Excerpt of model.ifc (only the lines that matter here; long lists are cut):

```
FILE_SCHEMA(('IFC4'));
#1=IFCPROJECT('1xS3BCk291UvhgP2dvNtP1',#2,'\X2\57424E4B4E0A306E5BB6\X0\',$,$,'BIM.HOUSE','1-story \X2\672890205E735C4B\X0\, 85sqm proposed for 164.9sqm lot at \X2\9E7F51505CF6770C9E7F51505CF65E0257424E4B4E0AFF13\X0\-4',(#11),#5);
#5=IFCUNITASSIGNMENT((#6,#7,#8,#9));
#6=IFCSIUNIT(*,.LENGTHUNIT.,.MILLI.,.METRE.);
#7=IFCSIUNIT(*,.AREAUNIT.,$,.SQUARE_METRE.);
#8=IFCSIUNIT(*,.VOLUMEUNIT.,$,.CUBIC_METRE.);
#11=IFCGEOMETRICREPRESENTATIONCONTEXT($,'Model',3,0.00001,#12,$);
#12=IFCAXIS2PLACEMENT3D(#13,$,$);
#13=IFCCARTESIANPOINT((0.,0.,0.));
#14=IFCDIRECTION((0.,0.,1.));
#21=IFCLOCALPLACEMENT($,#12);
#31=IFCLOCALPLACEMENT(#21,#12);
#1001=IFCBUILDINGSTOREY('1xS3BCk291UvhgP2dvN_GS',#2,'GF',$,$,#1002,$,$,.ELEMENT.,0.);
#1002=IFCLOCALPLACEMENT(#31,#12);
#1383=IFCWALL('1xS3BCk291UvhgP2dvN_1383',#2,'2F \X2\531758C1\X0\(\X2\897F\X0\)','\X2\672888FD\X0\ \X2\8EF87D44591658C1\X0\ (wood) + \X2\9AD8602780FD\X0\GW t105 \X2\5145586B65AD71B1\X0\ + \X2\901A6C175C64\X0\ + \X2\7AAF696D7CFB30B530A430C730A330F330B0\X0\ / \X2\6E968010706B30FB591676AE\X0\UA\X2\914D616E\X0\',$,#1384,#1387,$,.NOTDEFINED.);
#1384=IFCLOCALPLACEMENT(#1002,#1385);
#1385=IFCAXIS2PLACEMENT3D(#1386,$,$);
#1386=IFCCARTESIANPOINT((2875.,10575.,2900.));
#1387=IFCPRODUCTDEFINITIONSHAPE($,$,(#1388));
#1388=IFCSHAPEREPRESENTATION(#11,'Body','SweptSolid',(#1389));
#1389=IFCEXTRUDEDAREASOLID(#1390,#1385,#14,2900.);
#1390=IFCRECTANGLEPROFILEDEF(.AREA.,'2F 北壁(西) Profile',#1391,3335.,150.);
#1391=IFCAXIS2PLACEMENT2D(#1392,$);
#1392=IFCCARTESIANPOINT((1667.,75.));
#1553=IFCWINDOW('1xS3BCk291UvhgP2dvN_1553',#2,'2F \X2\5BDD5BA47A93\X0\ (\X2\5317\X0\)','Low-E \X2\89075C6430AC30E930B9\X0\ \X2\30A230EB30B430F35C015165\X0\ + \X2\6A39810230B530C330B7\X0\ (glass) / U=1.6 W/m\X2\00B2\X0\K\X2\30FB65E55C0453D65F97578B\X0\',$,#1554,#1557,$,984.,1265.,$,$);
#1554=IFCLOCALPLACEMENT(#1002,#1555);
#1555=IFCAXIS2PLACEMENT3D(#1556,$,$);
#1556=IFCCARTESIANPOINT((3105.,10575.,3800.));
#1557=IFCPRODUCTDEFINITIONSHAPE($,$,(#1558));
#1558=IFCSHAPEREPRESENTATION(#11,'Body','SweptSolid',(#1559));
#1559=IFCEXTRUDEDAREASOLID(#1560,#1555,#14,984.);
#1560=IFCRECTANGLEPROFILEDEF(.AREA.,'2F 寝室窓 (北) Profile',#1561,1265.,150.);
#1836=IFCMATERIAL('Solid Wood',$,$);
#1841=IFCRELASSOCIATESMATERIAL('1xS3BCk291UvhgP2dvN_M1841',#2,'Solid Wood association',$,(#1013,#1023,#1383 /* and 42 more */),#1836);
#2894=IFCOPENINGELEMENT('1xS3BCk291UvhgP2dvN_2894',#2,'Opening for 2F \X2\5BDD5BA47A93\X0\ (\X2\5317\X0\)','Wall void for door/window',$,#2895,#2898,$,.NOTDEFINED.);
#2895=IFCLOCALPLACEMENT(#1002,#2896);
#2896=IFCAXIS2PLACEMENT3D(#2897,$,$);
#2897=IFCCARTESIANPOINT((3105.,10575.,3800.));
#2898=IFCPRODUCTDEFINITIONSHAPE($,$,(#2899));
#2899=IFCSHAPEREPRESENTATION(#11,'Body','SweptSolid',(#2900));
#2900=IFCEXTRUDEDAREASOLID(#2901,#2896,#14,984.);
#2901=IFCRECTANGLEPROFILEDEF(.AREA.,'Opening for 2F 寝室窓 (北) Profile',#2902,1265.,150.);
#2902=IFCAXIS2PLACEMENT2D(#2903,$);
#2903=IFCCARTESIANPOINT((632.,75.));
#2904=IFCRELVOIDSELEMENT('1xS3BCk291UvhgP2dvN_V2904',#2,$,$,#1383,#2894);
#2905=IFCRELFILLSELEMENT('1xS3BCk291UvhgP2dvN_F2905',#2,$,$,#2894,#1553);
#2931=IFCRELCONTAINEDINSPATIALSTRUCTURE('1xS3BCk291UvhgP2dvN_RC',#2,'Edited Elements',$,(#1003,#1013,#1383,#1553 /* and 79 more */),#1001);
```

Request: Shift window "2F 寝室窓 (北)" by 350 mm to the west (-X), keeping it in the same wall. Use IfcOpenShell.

```python
import ifcopenshell
import ifcopenshell.api.geometry
import ifcopenshell.util.placement

model = ifcopenshell.open("model.ifc")

window = model.by_guid("1xS3BCk291UvhgP2dvN_1553")
opening = window.FillsVoids[0].RelatingOpeningElement
wall = opening.VoidsElements[0].RelatingBuildingElement

wall_matrix = ifcopenshell.util.placement.get_local_placement(wall.ObjectPlacement)
shift = wall_matrix[:3, 0] * -350.0
before = ifcopenshell.util.placement.get_local_placement(window.ObjectPlacement)[:3, 3].copy()

# The window is not placed relative to its opening, so move both.
for product in (opening, window):
    matrix = ifcopenshell.util.placement.get_local_placement(product.ObjectPlacement)
    matrix[:3, 3] += shift
    ifcopenshell.api.geometry.edit_object_placement(model, product=product, matrix=matrix, is_si=False)

after = ifcopenshell.util.placement.get_local_placement(window.ObjectPlacement)[:3, 3]
print("window moved by", (after - before).round(3) + 0.0)

model.write("model_v2.ifc")
```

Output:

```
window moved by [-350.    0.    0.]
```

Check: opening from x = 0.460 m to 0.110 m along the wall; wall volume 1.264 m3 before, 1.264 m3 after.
